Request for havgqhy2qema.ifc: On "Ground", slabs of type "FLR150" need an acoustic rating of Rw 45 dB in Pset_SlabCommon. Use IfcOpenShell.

First a look at what the model holds.

```python
import ifcopenshell
import ifcopenshell.util.element

model = ifcopenshell.open("havgqhy2qema.ifc")
print(model.schema)
storey = next(s for s in model.by_type("IfcBuildingStorey") if s.Name == "Ground")
slabs = [e for e in ifcopenshell.util.element.get_decomposition(storey) if e.is_a("IfcSlab")]
seen = {}
for e in slabs:
    element_type = ifcopenshell.util.element.get_type(e)
    key = (element_type.Name if element_type != e and element_type else None, ifcopenshell.util.element.get_pset(e, "Pset_SlabCommon", "AcousticRating"))
    seen[key] = seen.get(key, 0) + 1
for (name, value), count in sorted(seen.items(), key=str):
    print(count, "x", name, "|", value)
```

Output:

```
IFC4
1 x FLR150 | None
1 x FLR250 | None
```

```python
import ifcopenshell
import ifcopenshell.api.pset
import ifcopenshell.util.element

model = ifcopenshell.open("havgqhy2qema.ifc")

storey = next(s for s in model.by_type("IfcBuildingStorey") if s.Name == "Ground")
slabs = [e for e in ifcopenshell.util.element.get_decomposition(storey) if e.is_a("IfcSlab")]

count = 0
for e in slabs:
    element_type = ifcopenshell.util.element.get_type(e)
    if element_type in (None, e) or element_type.Name != "FLR150":
        continue
    # add_pset returns the element's existing set when there is one.
    pset = ifcopenshell.api.pset.add_pset(model, product=e, name="Pset_SlabCommon")
    ifcopenshell.api.pset.edit_pset(model, pset=pset, properties={"AcousticRating": "Rw 45 dB"})
    count += 1

print(count, "slabs updated")

model.write("havgqhy2qema_rev.ifc")
```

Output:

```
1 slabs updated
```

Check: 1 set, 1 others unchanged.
